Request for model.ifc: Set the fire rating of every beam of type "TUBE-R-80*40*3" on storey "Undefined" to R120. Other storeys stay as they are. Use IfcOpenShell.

First a look at what the model holds.

```python
import ifcopenshell
import ifcopenshell.util.element

model = ifcopenshell.open("model.ifc")
print(model.schema)
storey = next(s for s in model.by_type("IfcBuildingStorey") if s.Name == "Undefined")
beams = [e for e in ifcopenshell.util.element.get_decomposition(storey) if e.is_a("IfcBeam")]
seen = {}
for e in beams:
    element_type = ifcopenshell.util.element.get_type(e)
    key = (element_type.Name if element_type != e and element_type else None, ifcopenshell.util.element.get_pset(e, "Pset_BeamCommon", "FireRating"))
    seen[key] = seen.get(key, 0) + 1
for (name, value), count in sorted(seen.items(), key=str):
    print(count, "x", name, "|", value)
```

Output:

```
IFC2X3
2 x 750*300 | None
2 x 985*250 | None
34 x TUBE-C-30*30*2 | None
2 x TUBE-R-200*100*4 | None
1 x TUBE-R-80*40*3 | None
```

```python
import ifcopenshell
import ifcopenshell.api.pset
import ifcopenshell.util.element

model = ifcopenshell.open("model.ifc")

storey = next(s for s in model.by_type("IfcBuildingStorey") if s.Name == "Undefined")
beams = [e for e in ifcopenshell.util.element.get_decomposition(storey) if e.is_a("IfcBeam")]

count = 0
for e in beams:
    element_type = ifcopenshell.util.element.get_type(e)
    if element_type in (None, e) or element_type.Name != "TUBE-R-80*40*3":
        continue
    # add_pset returns the element's existing set when there is one.
    pset = ifcopenshell.api.pset.add_pset(model, product=e, name="Pset_BeamCommon")
    ifcopenshell.api.pset.edit_pset(model, pset=pset, properties={"FireRating": "R120"})
    count += 1

print(count, "beams updated")

model.write("model_updated.ifc")
```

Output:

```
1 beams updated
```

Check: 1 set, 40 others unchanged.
